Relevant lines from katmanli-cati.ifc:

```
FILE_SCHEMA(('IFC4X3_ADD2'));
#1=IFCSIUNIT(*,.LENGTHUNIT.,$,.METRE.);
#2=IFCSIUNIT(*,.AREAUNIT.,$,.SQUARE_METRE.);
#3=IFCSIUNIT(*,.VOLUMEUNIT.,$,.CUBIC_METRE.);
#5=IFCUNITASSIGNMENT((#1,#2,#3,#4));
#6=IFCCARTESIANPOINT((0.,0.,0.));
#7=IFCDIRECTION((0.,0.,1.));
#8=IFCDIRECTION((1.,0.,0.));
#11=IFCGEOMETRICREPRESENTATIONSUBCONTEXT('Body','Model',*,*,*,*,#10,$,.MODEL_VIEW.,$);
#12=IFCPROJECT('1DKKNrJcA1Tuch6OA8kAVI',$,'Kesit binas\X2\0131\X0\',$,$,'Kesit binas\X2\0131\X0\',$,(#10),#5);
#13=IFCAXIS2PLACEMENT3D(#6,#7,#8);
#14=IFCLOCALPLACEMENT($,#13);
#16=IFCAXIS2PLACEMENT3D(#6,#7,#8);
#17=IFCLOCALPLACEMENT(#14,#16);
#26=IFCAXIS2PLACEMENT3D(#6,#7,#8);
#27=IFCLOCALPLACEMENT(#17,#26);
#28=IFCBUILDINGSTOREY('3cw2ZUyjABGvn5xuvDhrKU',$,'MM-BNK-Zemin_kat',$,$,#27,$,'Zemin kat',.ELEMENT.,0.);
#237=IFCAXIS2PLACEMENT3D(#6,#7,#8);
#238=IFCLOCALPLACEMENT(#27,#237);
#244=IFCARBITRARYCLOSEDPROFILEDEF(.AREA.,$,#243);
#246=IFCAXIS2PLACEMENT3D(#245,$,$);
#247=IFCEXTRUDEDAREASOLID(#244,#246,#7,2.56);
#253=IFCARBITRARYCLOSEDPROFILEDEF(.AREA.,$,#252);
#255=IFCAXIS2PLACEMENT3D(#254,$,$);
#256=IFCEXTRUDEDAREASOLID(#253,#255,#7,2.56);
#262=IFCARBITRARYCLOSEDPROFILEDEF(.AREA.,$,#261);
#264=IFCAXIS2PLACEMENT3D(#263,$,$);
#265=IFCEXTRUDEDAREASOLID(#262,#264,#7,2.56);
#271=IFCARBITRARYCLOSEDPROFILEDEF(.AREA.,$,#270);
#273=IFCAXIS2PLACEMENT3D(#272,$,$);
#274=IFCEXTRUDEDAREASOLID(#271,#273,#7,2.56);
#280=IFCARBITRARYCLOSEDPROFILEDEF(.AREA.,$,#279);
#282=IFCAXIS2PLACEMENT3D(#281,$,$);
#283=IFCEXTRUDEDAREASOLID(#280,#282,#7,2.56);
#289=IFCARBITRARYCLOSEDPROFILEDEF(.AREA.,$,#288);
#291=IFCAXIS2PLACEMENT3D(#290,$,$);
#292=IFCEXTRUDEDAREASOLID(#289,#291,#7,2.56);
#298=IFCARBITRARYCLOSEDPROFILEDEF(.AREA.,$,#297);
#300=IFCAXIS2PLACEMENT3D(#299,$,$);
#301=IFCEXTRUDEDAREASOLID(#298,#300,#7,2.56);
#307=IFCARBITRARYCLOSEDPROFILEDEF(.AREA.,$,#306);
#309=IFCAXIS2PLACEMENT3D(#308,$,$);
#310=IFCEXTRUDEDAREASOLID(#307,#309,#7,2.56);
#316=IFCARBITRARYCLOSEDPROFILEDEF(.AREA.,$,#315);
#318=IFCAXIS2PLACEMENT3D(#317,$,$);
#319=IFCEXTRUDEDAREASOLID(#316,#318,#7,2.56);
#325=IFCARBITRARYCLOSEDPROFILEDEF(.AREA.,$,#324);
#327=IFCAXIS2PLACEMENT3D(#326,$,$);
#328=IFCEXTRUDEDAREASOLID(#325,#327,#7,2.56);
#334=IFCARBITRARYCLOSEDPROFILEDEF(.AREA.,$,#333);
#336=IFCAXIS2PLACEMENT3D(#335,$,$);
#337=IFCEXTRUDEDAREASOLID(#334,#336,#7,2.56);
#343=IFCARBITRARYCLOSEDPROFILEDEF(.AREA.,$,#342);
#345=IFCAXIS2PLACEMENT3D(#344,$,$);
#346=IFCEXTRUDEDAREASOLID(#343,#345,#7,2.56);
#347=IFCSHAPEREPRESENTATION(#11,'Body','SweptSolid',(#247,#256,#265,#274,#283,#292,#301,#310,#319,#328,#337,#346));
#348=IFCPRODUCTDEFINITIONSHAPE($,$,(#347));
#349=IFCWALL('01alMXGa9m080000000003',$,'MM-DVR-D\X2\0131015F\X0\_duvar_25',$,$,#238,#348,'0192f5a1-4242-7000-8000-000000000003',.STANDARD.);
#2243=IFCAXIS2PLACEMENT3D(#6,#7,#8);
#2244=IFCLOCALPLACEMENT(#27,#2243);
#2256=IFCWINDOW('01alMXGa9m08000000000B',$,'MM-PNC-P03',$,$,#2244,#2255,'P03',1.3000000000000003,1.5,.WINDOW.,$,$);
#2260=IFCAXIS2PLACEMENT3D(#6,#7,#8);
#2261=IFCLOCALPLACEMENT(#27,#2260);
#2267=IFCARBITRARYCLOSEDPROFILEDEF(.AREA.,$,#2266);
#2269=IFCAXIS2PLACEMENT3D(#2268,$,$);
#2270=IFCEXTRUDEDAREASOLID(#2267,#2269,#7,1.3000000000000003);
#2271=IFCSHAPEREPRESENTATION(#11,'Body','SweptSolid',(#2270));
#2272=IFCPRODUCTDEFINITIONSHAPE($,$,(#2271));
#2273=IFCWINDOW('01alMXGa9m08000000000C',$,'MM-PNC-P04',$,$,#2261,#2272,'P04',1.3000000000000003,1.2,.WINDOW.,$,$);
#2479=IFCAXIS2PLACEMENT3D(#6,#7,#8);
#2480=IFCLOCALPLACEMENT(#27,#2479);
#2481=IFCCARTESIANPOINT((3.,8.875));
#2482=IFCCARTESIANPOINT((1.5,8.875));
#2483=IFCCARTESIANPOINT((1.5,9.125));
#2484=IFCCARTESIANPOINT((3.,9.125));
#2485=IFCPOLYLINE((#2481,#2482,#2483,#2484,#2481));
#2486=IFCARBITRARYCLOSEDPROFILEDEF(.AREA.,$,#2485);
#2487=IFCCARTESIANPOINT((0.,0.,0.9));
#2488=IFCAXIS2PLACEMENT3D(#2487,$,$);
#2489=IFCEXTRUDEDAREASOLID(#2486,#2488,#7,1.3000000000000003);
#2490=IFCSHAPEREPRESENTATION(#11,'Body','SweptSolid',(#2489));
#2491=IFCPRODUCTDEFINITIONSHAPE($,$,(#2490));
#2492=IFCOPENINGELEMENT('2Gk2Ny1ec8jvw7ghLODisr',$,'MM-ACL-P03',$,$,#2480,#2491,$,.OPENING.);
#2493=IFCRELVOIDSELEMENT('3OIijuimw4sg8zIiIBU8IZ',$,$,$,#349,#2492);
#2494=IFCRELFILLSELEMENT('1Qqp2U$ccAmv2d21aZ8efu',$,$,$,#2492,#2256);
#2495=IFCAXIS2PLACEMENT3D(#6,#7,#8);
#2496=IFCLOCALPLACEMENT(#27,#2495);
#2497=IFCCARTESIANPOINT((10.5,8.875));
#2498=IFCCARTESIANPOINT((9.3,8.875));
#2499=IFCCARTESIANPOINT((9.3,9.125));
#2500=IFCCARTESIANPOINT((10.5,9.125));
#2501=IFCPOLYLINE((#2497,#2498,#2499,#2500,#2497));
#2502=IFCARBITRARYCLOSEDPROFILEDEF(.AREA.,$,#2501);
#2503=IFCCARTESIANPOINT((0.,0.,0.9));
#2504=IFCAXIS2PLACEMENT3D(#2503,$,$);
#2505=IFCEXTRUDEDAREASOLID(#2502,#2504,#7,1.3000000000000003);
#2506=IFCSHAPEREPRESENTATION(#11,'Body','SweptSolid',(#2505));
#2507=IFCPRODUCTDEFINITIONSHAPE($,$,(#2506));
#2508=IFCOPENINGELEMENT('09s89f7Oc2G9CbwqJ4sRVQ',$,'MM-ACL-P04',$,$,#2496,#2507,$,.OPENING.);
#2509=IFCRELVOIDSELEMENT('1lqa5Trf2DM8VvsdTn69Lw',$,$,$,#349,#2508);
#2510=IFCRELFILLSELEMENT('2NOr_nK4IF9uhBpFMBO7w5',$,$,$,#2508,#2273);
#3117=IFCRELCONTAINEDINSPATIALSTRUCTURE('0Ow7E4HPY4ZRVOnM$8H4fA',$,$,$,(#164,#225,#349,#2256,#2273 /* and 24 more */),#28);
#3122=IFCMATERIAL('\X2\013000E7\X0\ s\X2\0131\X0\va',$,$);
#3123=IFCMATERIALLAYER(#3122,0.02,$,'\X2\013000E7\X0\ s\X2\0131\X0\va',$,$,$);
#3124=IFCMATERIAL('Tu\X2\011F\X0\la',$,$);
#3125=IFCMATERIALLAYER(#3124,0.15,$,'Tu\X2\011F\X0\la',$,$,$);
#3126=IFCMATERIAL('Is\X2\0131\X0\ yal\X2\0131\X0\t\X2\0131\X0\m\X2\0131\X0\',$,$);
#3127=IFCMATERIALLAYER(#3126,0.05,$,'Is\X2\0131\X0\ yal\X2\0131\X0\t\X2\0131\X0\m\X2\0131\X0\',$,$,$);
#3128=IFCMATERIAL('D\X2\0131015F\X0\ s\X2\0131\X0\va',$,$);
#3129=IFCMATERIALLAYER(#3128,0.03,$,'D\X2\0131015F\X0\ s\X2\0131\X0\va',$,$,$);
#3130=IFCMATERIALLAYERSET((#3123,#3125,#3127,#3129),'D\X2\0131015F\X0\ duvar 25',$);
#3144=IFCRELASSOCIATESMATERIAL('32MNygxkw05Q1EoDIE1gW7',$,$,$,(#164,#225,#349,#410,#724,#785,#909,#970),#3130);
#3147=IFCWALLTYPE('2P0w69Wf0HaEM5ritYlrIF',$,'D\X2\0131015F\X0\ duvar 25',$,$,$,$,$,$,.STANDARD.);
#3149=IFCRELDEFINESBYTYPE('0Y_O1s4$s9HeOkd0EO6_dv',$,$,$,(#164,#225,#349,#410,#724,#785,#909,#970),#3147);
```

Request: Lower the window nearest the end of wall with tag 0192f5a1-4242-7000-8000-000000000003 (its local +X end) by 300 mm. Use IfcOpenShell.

```python
import numpy as np
import ifcopenshell
import ifcopenshell.api.geometry
import ifcopenshell.util.placement
import ifcopenshell.util.unit

model = ifcopenshell.open("katmanli-cati.ifc")
unit_scale = ifcopenshell.util.unit.calculate_unit_scale(model)

window = model.by_guid("01alMXGa9m08000000000C")
opening = window.FillsVoids[0].RelatingOpeningElement
dz = -0.3 / unit_scale

shift = np.array([0.0, 0.0, dz])
# The window is not placed relative to its opening, so move both.
for product in (opening, window):
    matrix = ifcopenshell.util.placement.get_local_placement(product.ObjectPlacement)
    matrix[:3, 3] += shift
    ifcopenshell.api.geometry.edit_object_placement(model, product=product, matrix=matrix, is_si=False)

print(f"moved by {dz * unit_scale:+.3f} m")

model.write("katmanli-cati-out.ifc")
```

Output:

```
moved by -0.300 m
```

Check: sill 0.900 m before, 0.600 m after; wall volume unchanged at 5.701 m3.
